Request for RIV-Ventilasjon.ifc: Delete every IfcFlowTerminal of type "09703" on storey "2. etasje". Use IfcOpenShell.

First a look at what the model holds.

```python
import ifcopenshell
import ifcopenshell.util.element

model = ifcopenshell.open("RIV-Ventilasjon.ifc")
print(model.schema)
storey = next(s for s in model.by_type("IfcBuildingStorey") if s.Name == "2. etasje")
terminals = [e for e in ifcopenshell.util.element.get_decomposition(storey) if e.is_a("IfcFlowTerminal")]
seen = {}
for e in terminals:
    element_type = ifcopenshell.util.element.get_type(e)
    name = element_type.Name if element_type not in (None, e) else None
    seen[name] = seen.get(name, 0) + 1
for name, count in sorted(seen.items(), key=str):
    print(count, "x", name)
```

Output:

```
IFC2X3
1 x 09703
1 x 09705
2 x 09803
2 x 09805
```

```python
import ifcopenshell
import ifcopenshell.api.root
import ifcopenshell.util.element

model = ifcopenshell.open("RIV-Ventilasjon.ifc")

storey = next(s for s in model.by_type("IfcBuildingStorey") if s.Name == "2. etasje")
terminals = [e for e in ifcopenshell.util.element.get_decomposition(storey) if e.is_a("IfcFlowTerminal")]
targets = [e for e in terminals if (t := ifcopenshell.util.element.get_type(e)) not in (None, e) and t.Name == "09703"]

for e in targets:
    ifcopenshell.api.root.remove_product(model, product=e)
print(len(targets), "removed")

model.write("RIV-Ventilasjon_rev.ifc")
```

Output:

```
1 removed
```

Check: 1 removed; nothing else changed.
